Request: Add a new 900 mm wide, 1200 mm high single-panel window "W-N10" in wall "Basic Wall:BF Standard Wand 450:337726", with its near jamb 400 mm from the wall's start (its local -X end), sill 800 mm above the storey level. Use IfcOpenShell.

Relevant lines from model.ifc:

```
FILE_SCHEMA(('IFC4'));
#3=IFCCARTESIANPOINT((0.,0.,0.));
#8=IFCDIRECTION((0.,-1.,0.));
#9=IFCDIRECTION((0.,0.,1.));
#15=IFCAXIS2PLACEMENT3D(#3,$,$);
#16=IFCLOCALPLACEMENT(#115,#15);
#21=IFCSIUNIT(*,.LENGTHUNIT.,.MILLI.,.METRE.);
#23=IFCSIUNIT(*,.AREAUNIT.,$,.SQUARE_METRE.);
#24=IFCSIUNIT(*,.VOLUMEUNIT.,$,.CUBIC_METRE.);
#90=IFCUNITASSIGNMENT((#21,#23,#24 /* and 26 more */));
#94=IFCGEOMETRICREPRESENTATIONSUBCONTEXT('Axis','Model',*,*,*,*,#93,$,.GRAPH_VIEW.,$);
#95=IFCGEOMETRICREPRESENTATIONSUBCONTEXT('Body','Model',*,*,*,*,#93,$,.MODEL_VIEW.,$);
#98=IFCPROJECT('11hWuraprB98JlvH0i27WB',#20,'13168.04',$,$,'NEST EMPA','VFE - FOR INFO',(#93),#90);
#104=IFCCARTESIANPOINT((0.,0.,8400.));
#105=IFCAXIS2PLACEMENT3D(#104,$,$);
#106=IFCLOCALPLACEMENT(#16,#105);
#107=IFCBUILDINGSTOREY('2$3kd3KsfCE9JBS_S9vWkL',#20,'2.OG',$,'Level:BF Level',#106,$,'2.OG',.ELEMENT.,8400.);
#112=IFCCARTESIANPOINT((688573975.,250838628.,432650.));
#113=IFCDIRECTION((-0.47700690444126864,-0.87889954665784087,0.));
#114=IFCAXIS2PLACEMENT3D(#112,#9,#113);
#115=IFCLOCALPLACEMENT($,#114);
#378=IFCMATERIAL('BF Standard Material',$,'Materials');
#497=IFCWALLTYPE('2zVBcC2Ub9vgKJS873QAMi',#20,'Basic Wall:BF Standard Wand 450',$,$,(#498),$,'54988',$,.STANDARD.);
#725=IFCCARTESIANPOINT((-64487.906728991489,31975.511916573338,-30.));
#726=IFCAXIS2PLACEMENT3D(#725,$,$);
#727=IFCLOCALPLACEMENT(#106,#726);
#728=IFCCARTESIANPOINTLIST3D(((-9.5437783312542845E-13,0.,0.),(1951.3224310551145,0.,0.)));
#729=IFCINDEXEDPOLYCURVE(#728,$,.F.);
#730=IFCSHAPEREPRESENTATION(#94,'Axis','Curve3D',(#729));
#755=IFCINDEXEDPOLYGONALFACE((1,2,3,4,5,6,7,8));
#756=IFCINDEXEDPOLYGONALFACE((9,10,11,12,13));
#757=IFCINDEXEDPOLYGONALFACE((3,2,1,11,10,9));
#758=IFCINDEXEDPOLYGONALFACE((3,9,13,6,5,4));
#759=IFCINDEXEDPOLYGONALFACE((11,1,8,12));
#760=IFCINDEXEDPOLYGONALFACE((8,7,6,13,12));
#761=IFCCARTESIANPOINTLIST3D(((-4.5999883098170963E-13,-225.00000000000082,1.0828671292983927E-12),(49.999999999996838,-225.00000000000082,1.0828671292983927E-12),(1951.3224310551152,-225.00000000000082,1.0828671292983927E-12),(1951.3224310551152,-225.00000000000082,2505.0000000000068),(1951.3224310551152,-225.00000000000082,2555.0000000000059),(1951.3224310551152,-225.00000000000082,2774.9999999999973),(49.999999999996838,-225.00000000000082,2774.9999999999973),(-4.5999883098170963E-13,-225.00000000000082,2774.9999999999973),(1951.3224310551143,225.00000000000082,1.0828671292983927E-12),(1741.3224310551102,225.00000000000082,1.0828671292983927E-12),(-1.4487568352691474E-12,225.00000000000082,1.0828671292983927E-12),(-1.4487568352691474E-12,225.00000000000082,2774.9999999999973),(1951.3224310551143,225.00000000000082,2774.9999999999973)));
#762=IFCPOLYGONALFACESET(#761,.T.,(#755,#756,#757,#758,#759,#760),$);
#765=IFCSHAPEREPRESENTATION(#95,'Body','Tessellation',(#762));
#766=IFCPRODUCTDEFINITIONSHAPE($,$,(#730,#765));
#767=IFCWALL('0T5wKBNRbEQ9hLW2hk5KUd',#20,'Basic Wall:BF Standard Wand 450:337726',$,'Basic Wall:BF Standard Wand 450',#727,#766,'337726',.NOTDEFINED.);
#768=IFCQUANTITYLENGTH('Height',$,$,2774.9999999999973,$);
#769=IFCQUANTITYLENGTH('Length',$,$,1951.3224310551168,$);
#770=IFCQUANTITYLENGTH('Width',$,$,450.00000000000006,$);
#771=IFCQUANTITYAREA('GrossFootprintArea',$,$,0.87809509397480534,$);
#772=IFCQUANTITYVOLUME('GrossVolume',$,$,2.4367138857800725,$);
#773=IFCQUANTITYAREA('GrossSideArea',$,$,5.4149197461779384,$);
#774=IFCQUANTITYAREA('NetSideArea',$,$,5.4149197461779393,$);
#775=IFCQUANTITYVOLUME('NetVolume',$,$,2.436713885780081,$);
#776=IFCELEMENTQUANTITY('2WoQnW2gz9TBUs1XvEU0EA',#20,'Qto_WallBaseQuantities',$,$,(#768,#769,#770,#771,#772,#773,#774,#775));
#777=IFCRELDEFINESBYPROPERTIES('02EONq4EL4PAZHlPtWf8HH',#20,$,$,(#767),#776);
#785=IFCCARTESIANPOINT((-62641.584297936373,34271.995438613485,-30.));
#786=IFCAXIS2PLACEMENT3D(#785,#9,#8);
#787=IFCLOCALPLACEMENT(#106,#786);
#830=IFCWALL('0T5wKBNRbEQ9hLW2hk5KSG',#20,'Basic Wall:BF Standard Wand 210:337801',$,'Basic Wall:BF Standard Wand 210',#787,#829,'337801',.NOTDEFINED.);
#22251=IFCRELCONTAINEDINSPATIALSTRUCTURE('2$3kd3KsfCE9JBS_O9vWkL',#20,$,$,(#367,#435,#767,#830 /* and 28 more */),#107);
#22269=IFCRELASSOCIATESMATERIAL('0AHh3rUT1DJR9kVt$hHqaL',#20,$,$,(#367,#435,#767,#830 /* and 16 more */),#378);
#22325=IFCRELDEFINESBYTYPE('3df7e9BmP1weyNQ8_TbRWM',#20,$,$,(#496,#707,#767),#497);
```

```python
import numpy as np
import ifcopenshell
import ifcopenshell.api.feature
import ifcopenshell.api.geometry
import ifcopenshell.api.pset
import ifcopenshell.api.root
import ifcopenshell.api.spatial
import ifcopenshell.geom
import ifcopenshell.util.element
import ifcopenshell.util.placement
import ifcopenshell.util.representation
import ifcopenshell.util.shape
import ifcopenshell.util.unit

model = ifcopenshell.open("model.ifc")
unit_scale = ifcopenshell.util.unit.calculate_unit_scale(model)
area_scale = ifcopenshell.util.unit.calculate_unit_scale(model, "AREAUNIT")
volume_scale = ifcopenshell.util.unit.calculate_unit_scale(model, "VOLUMEUNIT")
settings = ifcopenshell.geom.settings()


def volume(element):
    """Net volume in cubic metres, openings subtracted."""
    shape = ifcopenshell.geom.create_shape(settings, element)
    return ifcopenshell.util.shape.get_volume(shape.geometry)


wall = model.by_guid("0T5wKBNRbEQ9hLW2hk5KUd")
storey = ifcopenshell.util.element.get_container(wall, ifc_class="IfcBuildingStorey")
context = ifcopenshell.util.representation.get_context(model, "Model", "Body", "MODEL_VIEW")
before = volume(wall)

width, height, from_end, sill = 0.9, 1.2, 0.4, 0.8  # metres

# The wall runs along its own X axis, and the end named is its -X end.
wall_shape = ifcopenshell.geom.create_shape(settings, wall)
x, y, z = ifcopenshell.util.shape.get_vertices(wall_shape.geometry).T
start = x.min() + from_end
face, thickness = float(y.min()), float(y.max() - y.min())
wall_matrix = ifcopenshell.util.placement.get_local_placement(wall.ObjectPlacement)
level = ifcopenshell.util.placement.get_local_placement(storey.ObjectPlacement)[2, 3]


def in_wall(x, y):
    """Placement at x, y metres in the wall's axes, at sill height."""
    matrix = wall_matrix.copy()
    matrix[:, 3] = wall_matrix @ np.array([x / unit_scale, y / unit_scale, 0.0, 1.0])
    matrix[2, 3] = level + sill / unit_scale
    return matrix


# Opening: a box that overshoots both wall faces by 50 mm.
opening = ifcopenshell.api.root.create_entity(model, ifc_class="IfcOpeningElement", predefined_type="OPENING")
box = ifcopenshell.api.geometry.add_wall_representation(
    model, context=context, length=width, height=height, thickness=thickness + 0.1
)
ifcopenshell.api.geometry.assign_representation(model, product=opening, representation=box)
ifcopenshell.api.geometry.edit_object_placement(model, product=opening, matrix=in_wall(start, face - 0.05), is_si=False)
ifcopenshell.api.feature.add_feature(model, feature=opening, element=wall)

window = ifcopenshell.api.root.create_entity(model, ifc_class="IfcWindow", name="W-N10", predefined_type="WINDOW")
window.OverallWidth, window.OverallHeight = width / unit_scale, height / unit_scale
window.PartitioningType = "SINGLE_PANEL"
body = ifcopenshell.api.geometry.add_window_representation(
    model,
    context=context,
    overall_width=window.OverallWidth,
    overall_height=window.OverallHeight,
    partition_type="SINGLE_PANEL",
)
ifcopenshell.api.geometry.assign_representation(model, product=window, representation=body)
ifcopenshell.api.spatial.assign_container(model, products=[window], relating_structure=storey)
ifcopenshell.api.feature.add_filling(model, opening=opening, element=window)

# Centre the window in the wall's thickness.
ifcopenshell.api.geometry.edit_object_placement(model, product=window, matrix=in_wall(start, face), is_si=False)
window_shape = ifcopenshell.geom.create_shape(settings, window)
depth = ifcopenshell.util.shape.get_vertices(window_shape.geometry)[:, 1]
offset = face + thickness / 2 - (depth.min() + depth.max()) / 2
ifcopenshell.api.geometry.edit_object_placement(model, product=window, matrix=in_wall(start, offset), is_si=False)

after = volume(wall)

# Update the wall's stored quantities.
qto = model.by_id(ifcopenshell.util.element.get_pset(wall, "Qto_WallBaseQuantities", should_inherit=False)["id"])
ifcopenshell.api.pset.edit_qto(model, qto=qto, properties={
    "NetSideArea": after / thickness / area_scale,
    "NetVolume": after / volume_scale,
})

print(f"wall volume {before:.3f} -> {after:.3f} m3")

model.write("model_edited.ifc")
```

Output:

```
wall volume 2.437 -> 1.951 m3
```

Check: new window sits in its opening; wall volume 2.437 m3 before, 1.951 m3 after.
